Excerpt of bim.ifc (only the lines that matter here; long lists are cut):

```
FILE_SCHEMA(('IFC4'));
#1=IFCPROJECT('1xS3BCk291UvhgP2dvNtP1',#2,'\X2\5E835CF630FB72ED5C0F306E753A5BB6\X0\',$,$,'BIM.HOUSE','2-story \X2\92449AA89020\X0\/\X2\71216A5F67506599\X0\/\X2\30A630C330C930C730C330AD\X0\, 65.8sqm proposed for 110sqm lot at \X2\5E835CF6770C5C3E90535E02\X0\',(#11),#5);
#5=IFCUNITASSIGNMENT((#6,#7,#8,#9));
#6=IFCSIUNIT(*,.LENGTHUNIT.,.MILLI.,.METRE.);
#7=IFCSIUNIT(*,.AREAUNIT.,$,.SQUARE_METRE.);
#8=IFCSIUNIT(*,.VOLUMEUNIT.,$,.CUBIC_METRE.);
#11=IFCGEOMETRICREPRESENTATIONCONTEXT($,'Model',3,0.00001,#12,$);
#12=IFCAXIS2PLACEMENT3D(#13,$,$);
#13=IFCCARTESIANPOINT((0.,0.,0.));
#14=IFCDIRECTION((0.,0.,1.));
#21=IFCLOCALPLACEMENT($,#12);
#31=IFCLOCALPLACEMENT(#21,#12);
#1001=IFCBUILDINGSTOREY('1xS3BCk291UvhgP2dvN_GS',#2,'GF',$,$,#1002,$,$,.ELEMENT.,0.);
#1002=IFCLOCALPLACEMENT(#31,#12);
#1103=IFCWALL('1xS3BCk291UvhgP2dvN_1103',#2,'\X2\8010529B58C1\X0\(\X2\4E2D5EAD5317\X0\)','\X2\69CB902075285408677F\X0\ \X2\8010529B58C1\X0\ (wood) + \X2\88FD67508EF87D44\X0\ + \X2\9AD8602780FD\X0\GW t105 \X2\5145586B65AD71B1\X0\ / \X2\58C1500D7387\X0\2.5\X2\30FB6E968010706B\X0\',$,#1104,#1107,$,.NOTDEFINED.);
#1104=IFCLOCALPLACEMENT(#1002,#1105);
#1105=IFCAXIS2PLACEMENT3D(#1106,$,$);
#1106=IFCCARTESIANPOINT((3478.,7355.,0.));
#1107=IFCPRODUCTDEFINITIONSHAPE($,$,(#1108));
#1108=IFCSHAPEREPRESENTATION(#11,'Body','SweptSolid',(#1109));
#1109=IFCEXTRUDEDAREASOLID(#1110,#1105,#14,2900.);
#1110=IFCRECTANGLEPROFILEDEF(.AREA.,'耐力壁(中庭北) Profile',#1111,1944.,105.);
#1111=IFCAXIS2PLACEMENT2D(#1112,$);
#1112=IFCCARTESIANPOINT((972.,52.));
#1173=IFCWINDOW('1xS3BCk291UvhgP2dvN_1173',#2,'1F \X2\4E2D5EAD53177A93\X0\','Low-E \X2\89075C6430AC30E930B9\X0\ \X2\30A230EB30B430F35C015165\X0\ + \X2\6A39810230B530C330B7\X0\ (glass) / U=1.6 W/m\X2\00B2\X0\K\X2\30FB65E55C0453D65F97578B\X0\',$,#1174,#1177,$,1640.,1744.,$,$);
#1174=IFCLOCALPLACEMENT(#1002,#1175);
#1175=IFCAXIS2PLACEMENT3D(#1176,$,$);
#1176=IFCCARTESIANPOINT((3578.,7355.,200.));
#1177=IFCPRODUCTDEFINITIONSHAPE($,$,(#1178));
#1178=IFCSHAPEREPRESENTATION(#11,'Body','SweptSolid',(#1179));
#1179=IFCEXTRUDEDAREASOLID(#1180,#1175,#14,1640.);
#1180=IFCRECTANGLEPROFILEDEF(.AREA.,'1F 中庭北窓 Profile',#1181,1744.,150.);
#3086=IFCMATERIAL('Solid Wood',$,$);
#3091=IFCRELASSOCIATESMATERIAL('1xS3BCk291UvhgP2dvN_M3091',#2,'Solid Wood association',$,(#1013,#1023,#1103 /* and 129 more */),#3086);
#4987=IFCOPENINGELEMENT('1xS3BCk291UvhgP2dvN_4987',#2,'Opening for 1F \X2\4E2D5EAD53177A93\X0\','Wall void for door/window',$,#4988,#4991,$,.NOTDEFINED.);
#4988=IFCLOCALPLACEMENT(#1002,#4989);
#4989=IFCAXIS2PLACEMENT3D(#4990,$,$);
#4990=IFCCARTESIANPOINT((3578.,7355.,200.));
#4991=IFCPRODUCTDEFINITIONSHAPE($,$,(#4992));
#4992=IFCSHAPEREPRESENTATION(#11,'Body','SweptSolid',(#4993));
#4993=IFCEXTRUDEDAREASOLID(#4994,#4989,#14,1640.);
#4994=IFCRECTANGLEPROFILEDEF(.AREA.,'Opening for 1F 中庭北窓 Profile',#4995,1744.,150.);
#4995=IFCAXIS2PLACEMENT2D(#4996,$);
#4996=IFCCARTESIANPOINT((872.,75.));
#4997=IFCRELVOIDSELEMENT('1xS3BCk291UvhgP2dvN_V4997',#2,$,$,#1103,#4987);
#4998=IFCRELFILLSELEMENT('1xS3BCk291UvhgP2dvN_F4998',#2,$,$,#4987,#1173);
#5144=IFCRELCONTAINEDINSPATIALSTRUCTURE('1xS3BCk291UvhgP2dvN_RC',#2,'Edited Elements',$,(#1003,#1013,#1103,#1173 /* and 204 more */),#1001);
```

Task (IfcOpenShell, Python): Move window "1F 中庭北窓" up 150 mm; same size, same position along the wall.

```python
import numpy as np
import ifcopenshell
import ifcopenshell.api.geometry
import ifcopenshell.util.placement
import ifcopenshell.util.unit

model = ifcopenshell.open("bim.ifc")
unit_scale = ifcopenshell.util.unit.calculate_unit_scale(model)

window = model.by_guid("1xS3BCk291UvhgP2dvN_1173")
opening = window.FillsVoids[0].RelatingOpeningElement
dz = 150.0

shift = np.array([0.0, 0.0, dz])
# The window is not placed relative to its opening, so move both.
for product in (opening, window):
    matrix = ifcopenshell.util.placement.get_local_placement(product.ObjectPlacement)
    matrix[:3, 3] += shift
    ifcopenshell.api.geometry.edit_object_placement(model, product=product, matrix=matrix, is_si=False)

print(f"moved by {dz * unit_scale:+.3f} m")

model.write("bim-out.ifc")
```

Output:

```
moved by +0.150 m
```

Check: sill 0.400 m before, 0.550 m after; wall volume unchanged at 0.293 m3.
